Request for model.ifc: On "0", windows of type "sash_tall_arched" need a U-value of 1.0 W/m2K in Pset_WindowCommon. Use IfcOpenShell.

First a look at what the model holds.

```python
import ifcopenshell
import ifcopenshell.util.element

model = ifcopenshell.open("model.ifc")
print(model.schema)
storey = next(s for s in model.by_type("IfcBuildingStorey") if s.Name == "0")
windows = [e for e in ifcopenshell.util.element.get_decomposition(storey) if e.is_a("IfcWindow")]
seen = {}
for e in windows:
    element_type = ifcopenshell.util.element.get_type(e)
    key = (element_type.Name if element_type != e and element_type else None, ifcopenshell.util.element.get_pset(e, "Pset_WindowCommon", "ThermalTransmittance"))
    seen[key] = seen.get(key, 0) + 1
for (name, value), count in sorted(seen.items(), key=str):
    print(count, "x", name, "|", value)
```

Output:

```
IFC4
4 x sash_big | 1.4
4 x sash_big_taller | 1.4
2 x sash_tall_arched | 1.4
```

```python
import ifcopenshell
import ifcopenshell.api.pset
import ifcopenshell.util.element

model = ifcopenshell.open("model.ifc")

storey = next(s for s in model.by_type("IfcBuildingStorey") if s.Name == "0")
windows = [e for e in ifcopenshell.util.element.get_decomposition(storey) if e.is_a("IfcWindow")]

count = 0
for e in windows:
    element_type = ifcopenshell.util.element.get_type(e)
    if element_type in (None, e) or element_type.Name != "sash_tall_arched":
        continue
    # add_pset returns the element's existing set when there is one.
    pset = ifcopenshell.api.pset.add_pset(model, product=e, name="Pset_WindowCommon")
    ifcopenshell.api.pset.edit_pset(model, pset=pset, properties={"ThermalTransmittance": 1.0})
    count += 1

print(count, "windows updated")

model.write("model-out.ifc")
```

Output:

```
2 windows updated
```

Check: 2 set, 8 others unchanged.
